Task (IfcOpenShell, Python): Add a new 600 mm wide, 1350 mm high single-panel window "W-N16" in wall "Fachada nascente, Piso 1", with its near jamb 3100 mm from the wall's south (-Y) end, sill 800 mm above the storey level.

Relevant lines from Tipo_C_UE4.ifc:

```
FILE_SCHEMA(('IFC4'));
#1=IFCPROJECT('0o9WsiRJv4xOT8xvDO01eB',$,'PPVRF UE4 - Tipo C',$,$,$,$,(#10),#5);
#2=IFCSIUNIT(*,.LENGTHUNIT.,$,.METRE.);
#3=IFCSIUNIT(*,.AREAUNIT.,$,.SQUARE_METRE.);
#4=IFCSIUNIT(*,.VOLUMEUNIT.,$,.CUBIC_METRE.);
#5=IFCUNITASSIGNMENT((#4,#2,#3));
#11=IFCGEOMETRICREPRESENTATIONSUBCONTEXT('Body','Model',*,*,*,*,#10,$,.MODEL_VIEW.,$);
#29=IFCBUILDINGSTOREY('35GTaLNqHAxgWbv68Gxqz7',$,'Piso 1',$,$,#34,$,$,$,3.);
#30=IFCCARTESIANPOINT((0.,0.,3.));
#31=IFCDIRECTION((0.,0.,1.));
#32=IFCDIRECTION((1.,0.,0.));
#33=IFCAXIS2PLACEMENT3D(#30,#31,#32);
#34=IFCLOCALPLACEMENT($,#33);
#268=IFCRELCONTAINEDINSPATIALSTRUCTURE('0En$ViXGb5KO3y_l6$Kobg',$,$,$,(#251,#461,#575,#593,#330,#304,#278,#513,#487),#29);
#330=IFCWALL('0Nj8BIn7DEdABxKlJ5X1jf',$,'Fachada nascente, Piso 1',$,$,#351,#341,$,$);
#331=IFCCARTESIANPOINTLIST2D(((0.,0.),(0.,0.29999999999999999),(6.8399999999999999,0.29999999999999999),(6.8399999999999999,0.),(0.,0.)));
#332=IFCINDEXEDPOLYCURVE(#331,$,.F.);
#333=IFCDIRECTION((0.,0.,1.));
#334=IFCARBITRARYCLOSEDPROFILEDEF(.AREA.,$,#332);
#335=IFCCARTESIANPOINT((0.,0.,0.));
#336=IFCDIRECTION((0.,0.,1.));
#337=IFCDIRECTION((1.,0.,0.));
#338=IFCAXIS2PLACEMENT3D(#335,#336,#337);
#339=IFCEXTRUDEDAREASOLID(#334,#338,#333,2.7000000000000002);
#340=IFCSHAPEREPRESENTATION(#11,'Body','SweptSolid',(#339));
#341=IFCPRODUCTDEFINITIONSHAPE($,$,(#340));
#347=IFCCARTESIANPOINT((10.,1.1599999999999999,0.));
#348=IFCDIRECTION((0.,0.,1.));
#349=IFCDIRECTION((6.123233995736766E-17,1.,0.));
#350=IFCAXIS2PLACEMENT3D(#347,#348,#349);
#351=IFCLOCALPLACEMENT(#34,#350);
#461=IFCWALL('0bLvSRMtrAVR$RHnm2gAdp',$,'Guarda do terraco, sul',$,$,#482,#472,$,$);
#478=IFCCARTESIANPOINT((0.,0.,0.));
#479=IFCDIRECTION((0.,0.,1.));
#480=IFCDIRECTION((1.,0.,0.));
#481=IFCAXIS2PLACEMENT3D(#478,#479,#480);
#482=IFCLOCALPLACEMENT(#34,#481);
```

```python
import numpy as np
import ifcopenshell
import ifcopenshell.api.feature
import ifcopenshell.api.geometry
import ifcopenshell.api.root
import ifcopenshell.api.spatial
import ifcopenshell.geom
import ifcopenshell.util.element
import ifcopenshell.util.placement
import ifcopenshell.util.representation
import ifcopenshell.util.shape
import ifcopenshell.util.unit

model = ifcopenshell.open("Tipo_C_UE4.ifc")
unit_scale = ifcopenshell.util.unit.calculate_unit_scale(model)
settings = ifcopenshell.geom.settings()


def volume(element):
    """Net volume in cubic metres, openings subtracted."""
    shape = ifcopenshell.geom.create_shape(settings, element)
    return ifcopenshell.util.shape.get_volume(shape.geometry)


wall = model.by_id(330)
storey = ifcopenshell.util.element.get_container(wall, ifc_class="IfcBuildingStorey")
context = ifcopenshell.util.representation.get_context(model, "Model", "Body", "MODEL_VIEW")
before = volume(wall)

width, height, from_end, sill = 0.6, 1.35, 3.1, 0.8  # metres

# The wall runs along its own X axis, and the end named is its -X end.
wall_shape = ifcopenshell.geom.create_shape(settings, wall)
x, y, z = ifcopenshell.util.shape.get_vertices(wall_shape.geometry).T
start = x.min() + from_end
face, thickness = float(y.min()), float(y.max() - y.min())
wall_matrix = ifcopenshell.util.placement.get_local_placement(wall.ObjectPlacement)
level = ifcopenshell.util.placement.get_local_placement(storey.ObjectPlacement)[2, 3]


def in_wall(x, y):
    """Placement at x, y metres in the wall's axes, at sill height."""
    matrix = wall_matrix.copy()
    matrix[:, 3] = wall_matrix @ np.array([x / unit_scale, y / unit_scale, 0.0, 1.0])
    matrix[2, 3] = level + sill / unit_scale
    return matrix


# Opening: a box that overshoots both wall faces by 50 mm.
opening = ifcopenshell.api.root.create_entity(model, ifc_class="IfcOpeningElement", predefined_type="OPENING")
box = ifcopenshell.api.geometry.add_wall_representation(
    model, context=context, length=width, height=height, thickness=thickness + 0.1
)
ifcopenshell.api.geometry.assign_representation(model, product=opening, representation=box)
ifcopenshell.api.geometry.edit_object_placement(model, product=opening, matrix=in_wall(start, face - 0.05), is_si=False)
ifcopenshell.api.feature.add_feature(model, feature=opening, element=wall)

window = ifcopenshell.api.root.create_entity(model, ifc_class="IfcWindow", name="W-N16", predefined_type="WINDOW")
window.OverallWidth, window.OverallHeight = width / unit_scale, height / unit_scale
window.PartitioningType = "SINGLE_PANEL"
body = ifcopenshell.api.geometry.add_window_representation(
    model,
    context=context,
    overall_width=window.OverallWidth,
    overall_height=window.OverallHeight,
    partition_type="SINGLE_PANEL",
)
ifcopenshell.api.geometry.assign_representation(model, product=window, representation=body)
ifcopenshell.api.spatial.assign_container(model, products=[window], relating_structure=storey)
ifcopenshell.api.feature.add_filling(model, opening=opening, element=window)

# Centre the window in the wall's thickness.
ifcopenshell.api.geometry.edit_object_placement(model, product=window, matrix=in_wall(start, face), is_si=False)
window_shape = ifcopenshell.geom.create_shape(settings, window)
depth = ifcopenshell.util.shape.get_vertices(window_shape.geometry)[:, 1]
offset = face + thickness / 2 - (depth.min() + depth.max()) / 2
ifcopenshell.api.geometry.edit_object_placement(model, product=window, matrix=in_wall(start, offset), is_si=False)

after = volume(wall)

print(f"wall volume {before:.3f} -> {after:.3f} m3")

model.write("Tipo_C_UE4-out.ifc")
```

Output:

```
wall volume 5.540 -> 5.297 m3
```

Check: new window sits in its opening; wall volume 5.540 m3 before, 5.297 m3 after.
